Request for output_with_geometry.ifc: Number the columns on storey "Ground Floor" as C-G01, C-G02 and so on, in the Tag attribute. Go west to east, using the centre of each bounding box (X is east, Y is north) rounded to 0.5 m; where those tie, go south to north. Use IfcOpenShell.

First a look at what the model holds.

```python
import ifcopenshell
import ifcopenshell.util.element
import ifcopenshell.util.placement

model = ifcopenshell.open("output_with_geometry.ifc")
print(model.schema)
storey = next(s for s in model.by_type("IfcBuildingStorey") if s.Name == "Ground Floor")
columns = [e for e in ifcopenshell.util.element.get_decomposition(storey) if e.is_a("IfcColumn")]
for e in sorted(columns, key=lambda e: e.id()):
    origin = ifcopenshell.util.placement.get_local_placement(e.ObjectPlacement)[:3, 3]
    print(e.id(), e.Tag, e.Name, origin.round(2) + 0.0, sep=" | ")
```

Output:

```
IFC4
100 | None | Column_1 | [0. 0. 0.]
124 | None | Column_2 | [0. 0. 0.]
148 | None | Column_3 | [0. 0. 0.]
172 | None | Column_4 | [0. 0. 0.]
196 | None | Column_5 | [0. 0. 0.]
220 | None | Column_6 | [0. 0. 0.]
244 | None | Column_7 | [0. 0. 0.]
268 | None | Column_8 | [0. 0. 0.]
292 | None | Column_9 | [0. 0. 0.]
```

```python
import ifcopenshell
import ifcopenshell.geom
import ifcopenshell.util.element
import ifcopenshell.util.shape

model = ifcopenshell.open("output_with_geometry.ifc")
settings = ifcopenshell.geom.settings()
settings.set("use-world-coords", True)


def centre(element):
    shape = ifcopenshell.geom.create_shape(settings, element)
    return ifcopenshell.util.shape.get_bbox_centroid(shape.geometry)


storey = next(s for s in model.by_type("IfcBuildingStorey") if s.Name == "Ground Floor")
columns = [e for e in ifcopenshell.util.element.get_decomposition(storey) if e.is_a("IfcColumn")]

# Insertion points can sit at a corner or the storey origin, so sort by the geometry (in metres).
centres = {e: centre(e) for e in columns}
columns.sort(key=lambda e: (round(centres[e][0] / 0.5), centres[e][1]))

for i, e in enumerate(columns, start=1):
    number = f"C-G{i:02d}"
    e.Tag = number
    print(e.id(), number)

model.write("output_with_geometry_edited.ifc")
```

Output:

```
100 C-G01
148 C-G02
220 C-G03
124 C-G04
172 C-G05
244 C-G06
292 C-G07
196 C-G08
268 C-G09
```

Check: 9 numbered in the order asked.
